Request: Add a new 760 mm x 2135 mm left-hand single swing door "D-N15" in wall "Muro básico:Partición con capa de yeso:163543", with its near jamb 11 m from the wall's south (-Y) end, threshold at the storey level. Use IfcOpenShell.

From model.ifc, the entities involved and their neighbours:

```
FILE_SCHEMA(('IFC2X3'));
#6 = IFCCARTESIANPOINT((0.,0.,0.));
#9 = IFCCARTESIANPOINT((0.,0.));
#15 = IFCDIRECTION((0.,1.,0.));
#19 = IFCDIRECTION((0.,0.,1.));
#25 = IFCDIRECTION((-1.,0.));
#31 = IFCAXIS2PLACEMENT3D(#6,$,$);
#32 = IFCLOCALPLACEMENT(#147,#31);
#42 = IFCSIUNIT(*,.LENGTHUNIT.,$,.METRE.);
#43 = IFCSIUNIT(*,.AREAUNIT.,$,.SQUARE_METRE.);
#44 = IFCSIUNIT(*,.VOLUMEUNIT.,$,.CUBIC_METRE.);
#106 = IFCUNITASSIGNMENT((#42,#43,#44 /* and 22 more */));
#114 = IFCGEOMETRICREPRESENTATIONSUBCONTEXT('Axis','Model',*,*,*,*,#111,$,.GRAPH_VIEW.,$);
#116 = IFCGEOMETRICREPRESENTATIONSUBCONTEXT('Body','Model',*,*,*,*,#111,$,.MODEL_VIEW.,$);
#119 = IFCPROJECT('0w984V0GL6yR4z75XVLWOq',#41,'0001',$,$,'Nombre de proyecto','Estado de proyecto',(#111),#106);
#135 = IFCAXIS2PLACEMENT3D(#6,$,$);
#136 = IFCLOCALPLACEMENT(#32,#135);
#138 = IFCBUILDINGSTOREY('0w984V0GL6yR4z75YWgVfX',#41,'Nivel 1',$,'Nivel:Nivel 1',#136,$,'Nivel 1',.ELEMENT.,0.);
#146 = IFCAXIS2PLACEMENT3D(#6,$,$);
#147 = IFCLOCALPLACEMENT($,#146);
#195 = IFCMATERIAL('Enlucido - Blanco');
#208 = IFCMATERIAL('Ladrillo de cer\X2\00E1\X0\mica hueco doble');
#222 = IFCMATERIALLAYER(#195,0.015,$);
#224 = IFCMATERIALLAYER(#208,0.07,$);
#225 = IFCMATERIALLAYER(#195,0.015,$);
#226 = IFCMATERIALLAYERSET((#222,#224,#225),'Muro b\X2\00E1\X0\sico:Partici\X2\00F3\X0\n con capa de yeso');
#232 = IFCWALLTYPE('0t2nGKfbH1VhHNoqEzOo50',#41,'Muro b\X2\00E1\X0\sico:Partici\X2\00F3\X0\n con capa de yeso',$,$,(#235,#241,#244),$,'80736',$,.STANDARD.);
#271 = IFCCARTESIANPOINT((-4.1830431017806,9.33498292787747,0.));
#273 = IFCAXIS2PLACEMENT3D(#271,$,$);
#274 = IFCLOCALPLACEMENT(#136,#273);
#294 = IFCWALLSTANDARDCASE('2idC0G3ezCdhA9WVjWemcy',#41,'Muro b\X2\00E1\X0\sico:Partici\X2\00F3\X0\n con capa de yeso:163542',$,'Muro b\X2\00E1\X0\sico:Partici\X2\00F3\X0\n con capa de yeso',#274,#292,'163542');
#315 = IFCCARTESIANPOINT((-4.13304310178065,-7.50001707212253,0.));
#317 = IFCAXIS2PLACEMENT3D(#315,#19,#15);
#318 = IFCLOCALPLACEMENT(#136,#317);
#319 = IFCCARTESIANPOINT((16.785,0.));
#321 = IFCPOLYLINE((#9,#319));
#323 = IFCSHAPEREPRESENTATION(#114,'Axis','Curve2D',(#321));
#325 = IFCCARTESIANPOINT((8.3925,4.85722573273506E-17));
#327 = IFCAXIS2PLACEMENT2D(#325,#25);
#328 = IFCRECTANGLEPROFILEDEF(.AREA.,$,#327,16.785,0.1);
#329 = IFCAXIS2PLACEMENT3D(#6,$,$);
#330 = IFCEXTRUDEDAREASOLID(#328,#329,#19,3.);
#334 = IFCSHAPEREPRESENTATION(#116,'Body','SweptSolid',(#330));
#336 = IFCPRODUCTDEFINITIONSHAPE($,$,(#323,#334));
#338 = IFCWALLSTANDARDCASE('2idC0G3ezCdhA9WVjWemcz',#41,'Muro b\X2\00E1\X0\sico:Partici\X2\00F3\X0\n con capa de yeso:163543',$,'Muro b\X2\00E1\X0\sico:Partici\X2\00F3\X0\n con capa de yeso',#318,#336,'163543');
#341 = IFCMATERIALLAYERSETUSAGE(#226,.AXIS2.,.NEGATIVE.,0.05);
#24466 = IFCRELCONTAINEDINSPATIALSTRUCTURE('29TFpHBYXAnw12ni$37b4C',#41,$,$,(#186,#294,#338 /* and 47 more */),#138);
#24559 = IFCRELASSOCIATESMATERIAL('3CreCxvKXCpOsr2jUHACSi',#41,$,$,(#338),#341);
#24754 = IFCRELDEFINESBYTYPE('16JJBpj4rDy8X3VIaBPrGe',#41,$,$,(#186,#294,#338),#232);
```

```python
import numpy as np
import ifcopenshell
import ifcopenshell.api.feature
import ifcopenshell.api.geometry
import ifcopenshell.api.root
import ifcopenshell.api.spatial
import ifcopenshell.api.type
import ifcopenshell.geom
import ifcopenshell.util.element
import ifcopenshell.util.placement
import ifcopenshell.util.representation
import ifcopenshell.util.shape
import ifcopenshell.util.unit

model = ifcopenshell.open("model.ifc")
unit_scale = ifcopenshell.util.unit.calculate_unit_scale(model)
settings = ifcopenshell.geom.settings()


def volume(element):
    """Net volume in cubic metres, openings subtracted."""
    shape = ifcopenshell.geom.create_shape(settings, element)
    return ifcopenshell.util.shape.get_volume(shape.geometry)


wall = model.by_guid("2idC0G3ezCdhA9WVjWemcz")
storey = ifcopenshell.util.element.get_container(wall, ifc_class="IfcBuildingStorey")
context = ifcopenshell.util.representation.get_context(model, "Model", "Body", "MODEL_VIEW")
before = volume(wall)

width, height, from_end, sill = 0.76, 2.135, 11, 0.0  # metres

# The wall runs along its own X axis, and the end named is its -X end.
wall_shape = ifcopenshell.geom.create_shape(settings, wall)
x, y, z = ifcopenshell.util.shape.get_vertices(wall_shape.geometry).T
start = x.min() + from_end
face, thickness = float(y.min()), float(y.max() - y.min())
wall_matrix = ifcopenshell.util.placement.get_local_placement(wall.ObjectPlacement)
level = ifcopenshell.util.placement.get_local_placement(storey.ObjectPlacement)[2, 3]


def in_wall(x, y):
    """Placement at x, y metres in the wall's axes, at sill height."""
    matrix = wall_matrix.copy()
    matrix[:, 3] = wall_matrix @ np.array([x / unit_scale, y / unit_scale, 0.0, 1.0])
    matrix[2, 3] = level + sill / unit_scale
    return matrix


# Opening: a box that overshoots both wall faces by 50 mm.
opening = ifcopenshell.api.root.create_entity(model, ifc_class="IfcOpeningElement")
box = ifcopenshell.api.geometry.add_wall_representation(
    model, context=context, length=width, height=height, thickness=thickness + 0.1
)
ifcopenshell.api.geometry.assign_representation(model, product=opening, representation=box)
ifcopenshell.api.geometry.edit_object_placement(model, product=opening, matrix=in_wall(start, face - 0.05), is_si=False)
ifcopenshell.api.feature.add_feature(model, feature=opening, element=wall)

door = ifcopenshell.api.root.create_entity(model, ifc_class="IfcDoor", name="D-N15")
door.OverallWidth, door.OverallHeight = width / unit_scale, height / unit_scale
body = ifcopenshell.api.geometry.add_door_representation(
    model,
    context=context,
    overall_width=door.OverallWidth,
    overall_height=door.OverallHeight,
    operation_type="SINGLE_SWING_LEFT",
    lining_properties={"LiningDepth": thickness / unit_scale, "ThresholdDepth": thickness / unit_scale},
)
ifcopenshell.api.geometry.assign_representation(model, product=door, representation=body)
ifcopenshell.api.spatial.assign_container(model, products=[door], relating_structure=storey)
fills = ifcopenshell.api.feature.add_filling(model, opening=opening, element=door)
fills.OwnerHistory = door.OwnerHistory  # required in IFC2X3

# IFC2X3 keeps the operation on the door style.
style = ifcopenshell.api.root.create_entity(model, ifc_class="IfcDoorStyle", name="D-N15")
style.OperationType, style.ConstructionType = "SINGLE_SWING_LEFT", "NOTDEFINED"
style.ParameterTakesPrecedence = style.Sizeable = False
ifcopenshell.api.type.assign_type(model, related_objects=[door], relating_type=style)

# The lining spans the wall, so the door starts at the wall face.
ifcopenshell.api.geometry.edit_object_placement(model, product=door, matrix=in_wall(start, face), is_si=False)

after = volume(wall)

print(f"wall volume {before:.3f} -> {after:.3f} m3")

model.write("model-out.ifc")
```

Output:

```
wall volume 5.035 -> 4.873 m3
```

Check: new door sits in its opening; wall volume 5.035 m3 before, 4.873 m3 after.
